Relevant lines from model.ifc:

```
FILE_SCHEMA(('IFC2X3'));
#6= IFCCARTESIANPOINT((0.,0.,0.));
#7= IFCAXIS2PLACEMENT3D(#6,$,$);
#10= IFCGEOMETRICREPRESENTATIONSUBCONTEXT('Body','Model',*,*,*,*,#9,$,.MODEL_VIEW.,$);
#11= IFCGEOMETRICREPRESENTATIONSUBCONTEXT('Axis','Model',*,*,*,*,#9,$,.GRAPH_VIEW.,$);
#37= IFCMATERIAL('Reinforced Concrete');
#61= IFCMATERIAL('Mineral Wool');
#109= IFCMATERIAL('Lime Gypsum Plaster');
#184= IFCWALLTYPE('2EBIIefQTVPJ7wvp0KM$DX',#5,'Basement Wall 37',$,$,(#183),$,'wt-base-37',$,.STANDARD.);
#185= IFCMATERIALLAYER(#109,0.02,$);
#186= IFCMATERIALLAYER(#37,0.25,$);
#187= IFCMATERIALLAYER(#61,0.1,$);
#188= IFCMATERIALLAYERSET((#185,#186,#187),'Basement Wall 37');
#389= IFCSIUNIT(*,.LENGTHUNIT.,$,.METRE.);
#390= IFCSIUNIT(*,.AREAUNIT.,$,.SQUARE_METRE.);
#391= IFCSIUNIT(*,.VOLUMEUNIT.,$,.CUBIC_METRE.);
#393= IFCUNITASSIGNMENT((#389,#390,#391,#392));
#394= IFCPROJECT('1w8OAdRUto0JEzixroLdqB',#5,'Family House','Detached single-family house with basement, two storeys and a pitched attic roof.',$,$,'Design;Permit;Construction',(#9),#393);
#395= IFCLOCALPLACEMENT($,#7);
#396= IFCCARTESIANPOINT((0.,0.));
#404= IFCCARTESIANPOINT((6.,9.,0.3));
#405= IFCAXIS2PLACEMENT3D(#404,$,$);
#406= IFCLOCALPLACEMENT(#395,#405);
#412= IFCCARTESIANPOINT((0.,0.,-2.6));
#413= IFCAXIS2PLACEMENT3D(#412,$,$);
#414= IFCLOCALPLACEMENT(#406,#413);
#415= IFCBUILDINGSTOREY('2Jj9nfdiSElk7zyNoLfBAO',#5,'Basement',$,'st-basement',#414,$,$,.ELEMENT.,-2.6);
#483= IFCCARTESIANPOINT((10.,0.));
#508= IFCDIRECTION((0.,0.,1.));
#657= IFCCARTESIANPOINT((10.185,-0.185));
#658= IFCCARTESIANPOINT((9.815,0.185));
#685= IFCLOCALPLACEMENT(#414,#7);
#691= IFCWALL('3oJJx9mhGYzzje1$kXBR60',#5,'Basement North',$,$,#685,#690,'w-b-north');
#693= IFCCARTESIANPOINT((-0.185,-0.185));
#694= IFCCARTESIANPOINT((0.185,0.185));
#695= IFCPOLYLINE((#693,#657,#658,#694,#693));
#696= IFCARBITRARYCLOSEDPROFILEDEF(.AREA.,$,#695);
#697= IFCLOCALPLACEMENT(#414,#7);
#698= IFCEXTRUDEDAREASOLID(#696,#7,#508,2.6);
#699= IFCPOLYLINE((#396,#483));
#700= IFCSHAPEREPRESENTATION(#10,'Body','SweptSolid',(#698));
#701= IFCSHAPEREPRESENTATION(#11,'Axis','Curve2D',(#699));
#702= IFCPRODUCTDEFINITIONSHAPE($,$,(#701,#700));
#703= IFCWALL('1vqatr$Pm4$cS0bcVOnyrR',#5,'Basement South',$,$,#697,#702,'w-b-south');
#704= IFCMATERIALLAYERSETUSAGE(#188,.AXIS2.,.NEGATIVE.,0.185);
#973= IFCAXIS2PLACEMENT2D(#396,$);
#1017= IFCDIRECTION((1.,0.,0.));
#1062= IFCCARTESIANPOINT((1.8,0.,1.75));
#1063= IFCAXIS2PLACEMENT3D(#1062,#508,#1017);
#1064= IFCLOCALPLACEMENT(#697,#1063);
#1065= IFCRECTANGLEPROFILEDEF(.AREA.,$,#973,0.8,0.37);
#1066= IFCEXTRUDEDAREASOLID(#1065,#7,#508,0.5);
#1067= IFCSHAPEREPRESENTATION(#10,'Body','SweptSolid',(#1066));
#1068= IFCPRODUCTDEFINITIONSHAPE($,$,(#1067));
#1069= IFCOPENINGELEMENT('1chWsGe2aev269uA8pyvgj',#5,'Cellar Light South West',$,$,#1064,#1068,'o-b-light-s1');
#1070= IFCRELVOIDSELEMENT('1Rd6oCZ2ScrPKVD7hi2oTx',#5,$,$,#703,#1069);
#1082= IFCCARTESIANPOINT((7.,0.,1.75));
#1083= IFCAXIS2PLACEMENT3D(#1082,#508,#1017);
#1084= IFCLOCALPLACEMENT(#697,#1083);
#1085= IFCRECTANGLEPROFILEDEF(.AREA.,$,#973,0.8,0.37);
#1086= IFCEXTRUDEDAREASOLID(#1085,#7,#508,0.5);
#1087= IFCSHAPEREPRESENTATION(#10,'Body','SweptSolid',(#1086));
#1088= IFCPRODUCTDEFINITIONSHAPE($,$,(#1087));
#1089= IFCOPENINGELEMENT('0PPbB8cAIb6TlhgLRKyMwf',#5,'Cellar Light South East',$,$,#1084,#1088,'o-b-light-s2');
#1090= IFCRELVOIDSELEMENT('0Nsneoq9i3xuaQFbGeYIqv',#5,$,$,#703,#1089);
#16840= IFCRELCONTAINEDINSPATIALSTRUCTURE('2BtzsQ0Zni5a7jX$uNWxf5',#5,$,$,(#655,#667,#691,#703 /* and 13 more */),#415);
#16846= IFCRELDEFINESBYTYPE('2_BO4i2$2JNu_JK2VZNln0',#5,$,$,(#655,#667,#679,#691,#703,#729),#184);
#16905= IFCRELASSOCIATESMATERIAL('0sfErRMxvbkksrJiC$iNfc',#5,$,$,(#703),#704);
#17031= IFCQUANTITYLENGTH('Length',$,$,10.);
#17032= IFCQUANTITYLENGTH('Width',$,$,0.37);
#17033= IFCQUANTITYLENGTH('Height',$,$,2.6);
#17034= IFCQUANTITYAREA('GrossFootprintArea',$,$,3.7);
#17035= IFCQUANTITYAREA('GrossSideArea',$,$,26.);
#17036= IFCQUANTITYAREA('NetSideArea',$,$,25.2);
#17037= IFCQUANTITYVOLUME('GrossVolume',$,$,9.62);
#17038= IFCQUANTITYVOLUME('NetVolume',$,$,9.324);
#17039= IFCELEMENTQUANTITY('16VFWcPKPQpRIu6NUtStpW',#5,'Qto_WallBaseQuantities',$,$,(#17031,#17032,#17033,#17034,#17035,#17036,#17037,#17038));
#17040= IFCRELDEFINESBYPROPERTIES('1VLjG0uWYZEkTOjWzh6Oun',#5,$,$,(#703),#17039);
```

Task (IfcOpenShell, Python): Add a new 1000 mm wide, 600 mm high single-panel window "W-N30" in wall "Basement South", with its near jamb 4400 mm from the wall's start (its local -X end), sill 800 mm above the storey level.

```python
import numpy as np
import ifcopenshell
import ifcopenshell.api.feature
import ifcopenshell.api.geometry
import ifcopenshell.api.pset
import ifcopenshell.api.root
import ifcopenshell.api.spatial
import ifcopenshell.api.type
import ifcopenshell.geom
import ifcopenshell.util.element
import ifcopenshell.util.placement
import ifcopenshell.util.representation
import ifcopenshell.util.shape
import ifcopenshell.util.unit

model = ifcopenshell.open("model.ifc")
unit_scale = ifcopenshell.util.unit.calculate_unit_scale(model)
area_scale = ifcopenshell.util.unit.calculate_unit_scale(model, "AREAUNIT")
volume_scale = ifcopenshell.util.unit.calculate_unit_scale(model, "VOLUMEUNIT")
settings = ifcopenshell.geom.settings()


def volume(element):
    """Net volume in cubic metres, openings subtracted."""
    shape = ifcopenshell.geom.create_shape(settings, element)
    return ifcopenshell.util.shape.get_volume(shape.geometry)


wall = model.by_guid("1vqatr$Pm4$cS0bcVOnyrR")
storey = ifcopenshell.util.element.get_container(wall, ifc_class="IfcBuildingStorey")
context = ifcopenshell.util.representation.get_context(model, "Model", "Body", "MODEL_VIEW")
before = volume(wall)

width, height, from_end, sill = 1, 0.6, 4.4, 0.8  # metres

# The wall runs along its own X axis, and the end named is its -X end.
wall_shape = ifcopenshell.geom.create_shape(settings, wall)
x, y, z = ifcopenshell.util.shape.get_vertices(wall_shape.geometry).T
start = x.min() + from_end
face, thickness = float(y.min()), float(y.max() - y.min())
wall_matrix = ifcopenshell.util.placement.get_local_placement(wall.ObjectPlacement)
level = ifcopenshell.util.placement.get_local_placement(storey.ObjectPlacement)[2, 3]


def in_wall(x, y):
    """Placement at x, y metres in the wall's axes, at sill height."""
    matrix = wall_matrix.copy()
    matrix[:, 3] = wall_matrix @ np.array([x / unit_scale, y / unit_scale, 0.0, 1.0])
    matrix[2, 3] = level + sill / unit_scale
    return matrix


# Opening: a box that overshoots both wall faces by 50 mm.
opening = ifcopenshell.api.root.create_entity(model, ifc_class="IfcOpeningElement")
box = ifcopenshell.api.geometry.add_wall_representation(
    model, context=context, length=width, height=height, thickness=thickness + 0.1
)
ifcopenshell.api.geometry.assign_representation(model, product=opening, representation=box)
ifcopenshell.api.geometry.edit_object_placement(model, product=opening, matrix=in_wall(start, face - 0.05), is_si=False)
ifcopenshell.api.feature.add_feature(model, feature=opening, element=wall)

window = ifcopenshell.api.root.create_entity(model, ifc_class="IfcWindow", name="W-N30")
window.OverallWidth, window.OverallHeight = width / unit_scale, height / unit_scale
body = ifcopenshell.api.geometry.add_window_representation(
    model,
    context=context,
    overall_width=window.OverallWidth,
    overall_height=window.OverallHeight,
    partition_type="SINGLE_PANEL",
)
ifcopenshell.api.geometry.assign_representation(model, product=window, representation=body)
ifcopenshell.api.spatial.assign_container(model, products=[window], relating_structure=storey)
fills = ifcopenshell.api.feature.add_filling(model, opening=opening, element=window)
fills.OwnerHistory = window.OwnerHistory  # required in IFC2X3

# IFC2X3 keeps the operation on the window style.
style = ifcopenshell.api.root.create_entity(model, ifc_class="IfcWindowStyle", name="W-N30")
style.OperationType, style.ConstructionType = "SINGLE_PANEL", "NOTDEFINED"
style.ParameterTakesPrecedence = style.Sizeable = False
ifcopenshell.api.type.assign_type(model, related_objects=[window], relating_type=style)

# Centre the window in the wall's thickness.
ifcopenshell.api.geometry.edit_object_placement(model, product=window, matrix=in_wall(start, face), is_si=False)
window_shape = ifcopenshell.geom.create_shape(settings, window)
depth = ifcopenshell.util.shape.get_vertices(window_shape.geometry)[:, 1]
offset = face + thickness / 2 - (depth.min() + depth.max()) / 2
ifcopenshell.api.geometry.edit_object_placement(model, product=window, matrix=in_wall(start, offset), is_si=False)

after = volume(wall)

# Update the wall's stored quantities.
qto = model.by_id(ifcopenshell.util.element.get_pset(wall, "Qto_WallBaseQuantities", should_inherit=False)["id"])
ifcopenshell.api.pset.edit_qto(model, qto=qto, properties={
    "NetSideArea": after / thickness / area_scale,
    "NetVolume": after / volume_scale,
})

print(f"wall volume {before:.3f} -> {after:.3f} m3")

model.write("model_updated.ifc")
```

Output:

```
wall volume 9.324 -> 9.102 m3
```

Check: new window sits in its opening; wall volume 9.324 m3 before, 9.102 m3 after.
